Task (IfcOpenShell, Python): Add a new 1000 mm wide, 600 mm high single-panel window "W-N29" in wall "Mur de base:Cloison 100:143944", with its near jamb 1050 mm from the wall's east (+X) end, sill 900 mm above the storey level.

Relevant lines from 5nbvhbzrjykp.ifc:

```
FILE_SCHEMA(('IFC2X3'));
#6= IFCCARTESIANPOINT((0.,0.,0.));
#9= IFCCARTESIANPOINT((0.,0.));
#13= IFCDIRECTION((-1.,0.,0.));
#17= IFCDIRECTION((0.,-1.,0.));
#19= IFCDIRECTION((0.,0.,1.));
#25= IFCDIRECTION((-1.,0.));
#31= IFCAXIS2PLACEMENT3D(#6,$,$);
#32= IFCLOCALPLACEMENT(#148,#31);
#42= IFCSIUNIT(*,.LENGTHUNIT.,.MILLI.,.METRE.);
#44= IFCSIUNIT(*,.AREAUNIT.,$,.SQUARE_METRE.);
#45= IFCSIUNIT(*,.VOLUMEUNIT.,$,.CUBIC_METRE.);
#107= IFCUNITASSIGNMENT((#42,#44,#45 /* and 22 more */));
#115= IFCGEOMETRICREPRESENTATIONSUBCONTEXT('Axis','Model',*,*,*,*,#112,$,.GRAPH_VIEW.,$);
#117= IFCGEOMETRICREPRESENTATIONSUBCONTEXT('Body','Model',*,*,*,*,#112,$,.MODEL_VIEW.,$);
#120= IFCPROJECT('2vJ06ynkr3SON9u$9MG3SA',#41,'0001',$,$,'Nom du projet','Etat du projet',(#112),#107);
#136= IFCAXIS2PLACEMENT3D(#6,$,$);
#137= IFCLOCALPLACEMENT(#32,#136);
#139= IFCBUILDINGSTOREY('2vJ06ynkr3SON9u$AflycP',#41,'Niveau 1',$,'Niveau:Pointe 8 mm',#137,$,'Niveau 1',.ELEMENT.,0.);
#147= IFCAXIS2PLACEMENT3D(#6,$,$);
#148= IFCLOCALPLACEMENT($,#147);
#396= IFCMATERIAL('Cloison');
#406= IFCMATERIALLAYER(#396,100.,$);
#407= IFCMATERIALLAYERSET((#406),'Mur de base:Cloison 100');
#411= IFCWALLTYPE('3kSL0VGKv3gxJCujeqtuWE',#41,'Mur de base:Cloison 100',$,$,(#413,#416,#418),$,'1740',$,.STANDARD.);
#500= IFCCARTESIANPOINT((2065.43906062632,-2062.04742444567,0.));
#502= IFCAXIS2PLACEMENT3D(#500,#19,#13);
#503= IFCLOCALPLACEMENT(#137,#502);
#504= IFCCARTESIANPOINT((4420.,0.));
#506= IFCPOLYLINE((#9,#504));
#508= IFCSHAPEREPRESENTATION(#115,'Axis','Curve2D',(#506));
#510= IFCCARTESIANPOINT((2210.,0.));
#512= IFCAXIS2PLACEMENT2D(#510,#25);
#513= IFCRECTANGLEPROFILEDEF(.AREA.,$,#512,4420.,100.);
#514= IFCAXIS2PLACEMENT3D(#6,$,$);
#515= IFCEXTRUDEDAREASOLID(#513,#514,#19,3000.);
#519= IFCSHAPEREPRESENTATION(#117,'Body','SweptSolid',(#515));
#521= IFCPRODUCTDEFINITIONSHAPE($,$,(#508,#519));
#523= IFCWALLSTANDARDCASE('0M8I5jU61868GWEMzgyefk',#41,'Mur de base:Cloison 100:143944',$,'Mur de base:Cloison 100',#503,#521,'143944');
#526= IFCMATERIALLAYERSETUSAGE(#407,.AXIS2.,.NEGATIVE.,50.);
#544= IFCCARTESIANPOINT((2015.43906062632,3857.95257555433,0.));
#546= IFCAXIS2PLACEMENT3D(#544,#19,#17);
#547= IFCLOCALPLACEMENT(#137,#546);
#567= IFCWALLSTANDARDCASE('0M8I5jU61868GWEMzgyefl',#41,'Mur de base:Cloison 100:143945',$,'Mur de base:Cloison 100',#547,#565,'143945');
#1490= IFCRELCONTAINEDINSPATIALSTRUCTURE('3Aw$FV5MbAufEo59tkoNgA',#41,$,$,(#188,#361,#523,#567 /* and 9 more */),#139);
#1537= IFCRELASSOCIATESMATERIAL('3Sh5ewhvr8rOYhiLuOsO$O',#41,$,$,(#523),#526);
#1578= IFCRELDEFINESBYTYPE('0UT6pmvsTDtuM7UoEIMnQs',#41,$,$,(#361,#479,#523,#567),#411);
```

```python
import numpy as np
import ifcopenshell
import ifcopenshell.api.feature
import ifcopenshell.api.geometry
import ifcopenshell.api.root
import ifcopenshell.api.spatial
import ifcopenshell.api.type
import ifcopenshell.geom
import ifcopenshell.util.element
import ifcopenshell.util.placement
import ifcopenshell.util.representation
import ifcopenshell.util.shape
import ifcopenshell.util.unit

model = ifcopenshell.open("5nbvhbzrjykp.ifc")
unit_scale = ifcopenshell.util.unit.calculate_unit_scale(model)
settings = ifcopenshell.geom.settings()


def volume(element):
    """Net volume in cubic metres, openings subtracted."""
    shape = ifcopenshell.geom.create_shape(settings, element)
    return ifcopenshell.util.shape.get_volume(shape.geometry)


wall = model.by_guid("0M8I5jU61868GWEMzgyefk")
storey = ifcopenshell.util.element.get_container(wall, ifc_class="IfcBuildingStorey")
context = ifcopenshell.util.representation.get_context(model, "Model", "Body", "MODEL_VIEW")
before = volume(wall)

width, height, from_end, sill = 1, 0.6, 1.05, 0.9  # metres

# The wall runs along its own X axis, and the end named is its -X end.
wall_shape = ifcopenshell.geom.create_shape(settings, wall)
x, y, z = ifcopenshell.util.shape.get_vertices(wall_shape.geometry).T
start = x.min() + from_end
face, thickness = float(y.min()), float(y.max() - y.min())
wall_matrix = ifcopenshell.util.placement.get_local_placement(wall.ObjectPlacement)
level = ifcopenshell.util.placement.get_local_placement(storey.ObjectPlacement)[2, 3]


def in_wall(x, y):
    """Placement at x, y metres in the wall's axes, at sill height."""
    matrix = wall_matrix.copy()
    matrix[:, 3] = wall_matrix @ np.array([x / unit_scale, y / unit_scale, 0.0, 1.0])
    matrix[2, 3] = level + sill / unit_scale
    return matrix


# Opening: a box that overshoots both wall faces by 50 mm.
opening = ifcopenshell.api.root.create_entity(model, ifc_class="IfcOpeningElement")
box = ifcopenshell.api.geometry.add_wall_representation(
    model, context=context, length=width, height=height, thickness=thickness + 0.1
)
ifcopenshell.api.geometry.assign_representation(model, product=opening, representation=box)
ifcopenshell.api.geometry.edit_object_placement(model, product=opening, matrix=in_wall(start, face - 0.05), is_si=False)
ifcopenshell.api.feature.add_feature(model, feature=opening, element=wall)

window = ifcopenshell.api.root.create_entity(model, ifc_class="IfcWindow", name="W-N29")
window.OverallWidth, window.OverallHeight = width / unit_scale, height / unit_scale
body = ifcopenshell.api.geometry.add_window_representation(
    model,
    context=context,
    overall_width=window.OverallWidth,
    overall_height=window.OverallHeight,
    partition_type="SINGLE_PANEL",
)
ifcopenshell.api.geometry.assign_representation(model, product=window, representation=body)
ifcopenshell.api.spatial.assign_container(model, products=[window], relating_structure=storey)
fills = ifcopenshell.api.feature.add_filling(model, opening=opening, element=window)
fills.OwnerHistory = window.OwnerHistory  # required in IFC2X3

# IFC2X3 keeps the operation on the window style.
style = ifcopenshell.api.root.create_entity(model, ifc_class="IfcWindowStyle", name="W-N29")
style.OperationType, style.ConstructionType = "SINGLE_PANEL", "NOTDEFINED"
style.ParameterTakesPrecedence = style.Sizeable = False
ifcopenshell.api.type.assign_type(model, related_objects=[window], relating_type=style)

# Centre the window in the wall's thickness.
ifcopenshell.api.geometry.edit_object_placement(model, product=window, matrix=in_wall(start, face), is_si=False)
window_shape = ifcopenshell.geom.create_shape(settings, window)
depth = ifcopenshell.util.shape.get_vertices(window_shape.geometry)[:, 1]
offset = face + thickness / 2 - (depth.min() + depth.max()) / 2
ifcopenshell.api.geometry.edit_object_placement(model, product=window, matrix=in_wall(start, offset), is_si=False)

after = volume(wall)

print(f"wall volume {before:.3f} -> {after:.3f} m3")

model.write("5nbvhbzrjykp_v2.ifc")
```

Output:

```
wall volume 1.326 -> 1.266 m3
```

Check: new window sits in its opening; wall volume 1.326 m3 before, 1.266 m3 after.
